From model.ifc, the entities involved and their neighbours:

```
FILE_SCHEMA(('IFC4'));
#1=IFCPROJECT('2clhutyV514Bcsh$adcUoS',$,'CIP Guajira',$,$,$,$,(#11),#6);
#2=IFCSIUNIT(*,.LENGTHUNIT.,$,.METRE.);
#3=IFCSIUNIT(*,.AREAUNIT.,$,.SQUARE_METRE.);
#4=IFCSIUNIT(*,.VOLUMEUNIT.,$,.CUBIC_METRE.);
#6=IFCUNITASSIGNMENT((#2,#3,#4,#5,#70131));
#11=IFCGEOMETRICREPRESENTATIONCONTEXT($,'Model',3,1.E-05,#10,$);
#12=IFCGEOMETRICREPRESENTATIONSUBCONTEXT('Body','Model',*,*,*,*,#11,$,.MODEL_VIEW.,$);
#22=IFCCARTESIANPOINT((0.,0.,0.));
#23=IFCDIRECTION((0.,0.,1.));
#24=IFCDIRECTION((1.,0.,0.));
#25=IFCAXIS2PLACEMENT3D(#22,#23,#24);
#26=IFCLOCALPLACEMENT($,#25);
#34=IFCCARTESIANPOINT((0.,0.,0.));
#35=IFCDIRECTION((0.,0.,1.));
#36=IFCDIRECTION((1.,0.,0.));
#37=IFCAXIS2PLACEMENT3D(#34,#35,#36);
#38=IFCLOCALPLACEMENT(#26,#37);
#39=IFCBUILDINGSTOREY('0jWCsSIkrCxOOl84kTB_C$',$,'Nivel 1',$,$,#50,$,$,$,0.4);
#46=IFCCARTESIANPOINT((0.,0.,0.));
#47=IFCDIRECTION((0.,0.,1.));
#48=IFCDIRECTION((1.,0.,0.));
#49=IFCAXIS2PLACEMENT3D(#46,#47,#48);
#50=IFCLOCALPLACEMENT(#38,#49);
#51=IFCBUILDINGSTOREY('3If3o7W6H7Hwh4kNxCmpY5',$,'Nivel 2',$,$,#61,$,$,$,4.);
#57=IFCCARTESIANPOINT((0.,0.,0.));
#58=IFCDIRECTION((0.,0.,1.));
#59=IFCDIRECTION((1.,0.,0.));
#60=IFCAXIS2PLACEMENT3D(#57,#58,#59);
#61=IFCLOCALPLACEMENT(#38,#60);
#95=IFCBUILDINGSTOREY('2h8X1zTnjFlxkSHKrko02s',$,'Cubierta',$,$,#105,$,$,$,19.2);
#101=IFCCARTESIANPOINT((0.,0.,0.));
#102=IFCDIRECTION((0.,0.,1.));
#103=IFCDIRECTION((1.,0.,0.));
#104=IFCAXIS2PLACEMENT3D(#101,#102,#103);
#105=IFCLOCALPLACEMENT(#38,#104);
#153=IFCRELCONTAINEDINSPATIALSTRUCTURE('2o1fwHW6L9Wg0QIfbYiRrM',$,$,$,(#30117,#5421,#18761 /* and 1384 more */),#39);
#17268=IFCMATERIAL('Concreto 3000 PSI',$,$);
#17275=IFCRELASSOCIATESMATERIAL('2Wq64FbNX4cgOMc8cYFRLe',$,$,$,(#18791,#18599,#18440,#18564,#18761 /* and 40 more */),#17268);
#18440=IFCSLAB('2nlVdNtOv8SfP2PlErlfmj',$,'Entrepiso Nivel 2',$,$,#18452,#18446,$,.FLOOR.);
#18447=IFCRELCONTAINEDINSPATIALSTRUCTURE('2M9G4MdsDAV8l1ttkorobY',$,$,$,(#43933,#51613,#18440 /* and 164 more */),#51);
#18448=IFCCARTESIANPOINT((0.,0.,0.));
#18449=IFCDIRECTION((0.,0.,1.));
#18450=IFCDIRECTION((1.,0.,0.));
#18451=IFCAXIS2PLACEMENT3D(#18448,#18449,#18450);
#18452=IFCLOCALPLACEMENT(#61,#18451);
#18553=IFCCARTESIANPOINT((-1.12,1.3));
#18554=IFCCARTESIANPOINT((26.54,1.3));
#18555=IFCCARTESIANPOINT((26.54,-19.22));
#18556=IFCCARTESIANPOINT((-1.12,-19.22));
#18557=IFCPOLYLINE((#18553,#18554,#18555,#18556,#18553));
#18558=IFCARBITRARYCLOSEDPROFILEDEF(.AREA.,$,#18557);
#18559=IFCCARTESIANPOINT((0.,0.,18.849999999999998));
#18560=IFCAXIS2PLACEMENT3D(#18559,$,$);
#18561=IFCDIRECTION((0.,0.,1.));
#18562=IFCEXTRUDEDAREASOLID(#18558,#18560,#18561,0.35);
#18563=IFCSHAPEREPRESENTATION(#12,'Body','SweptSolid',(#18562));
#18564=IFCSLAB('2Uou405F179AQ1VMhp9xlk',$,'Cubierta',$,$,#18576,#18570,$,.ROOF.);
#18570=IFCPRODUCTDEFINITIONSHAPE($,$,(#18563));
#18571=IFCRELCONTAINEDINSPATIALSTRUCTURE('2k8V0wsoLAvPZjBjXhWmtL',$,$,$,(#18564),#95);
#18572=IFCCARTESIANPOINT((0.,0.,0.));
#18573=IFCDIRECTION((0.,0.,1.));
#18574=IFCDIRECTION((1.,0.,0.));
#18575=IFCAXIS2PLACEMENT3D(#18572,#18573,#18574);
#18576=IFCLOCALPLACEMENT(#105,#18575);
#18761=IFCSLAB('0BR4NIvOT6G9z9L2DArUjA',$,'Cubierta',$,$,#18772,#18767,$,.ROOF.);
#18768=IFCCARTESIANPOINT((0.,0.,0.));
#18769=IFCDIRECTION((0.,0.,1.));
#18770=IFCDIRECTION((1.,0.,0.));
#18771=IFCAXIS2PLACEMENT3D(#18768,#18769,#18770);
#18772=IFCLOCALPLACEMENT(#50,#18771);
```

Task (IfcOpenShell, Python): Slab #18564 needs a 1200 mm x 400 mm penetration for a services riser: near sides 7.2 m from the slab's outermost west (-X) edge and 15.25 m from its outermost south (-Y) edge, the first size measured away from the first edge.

```python
import numpy as np
import ifcopenshell
import ifcopenshell.api.feature
import ifcopenshell.api.geometry
import ifcopenshell.api.root
import ifcopenshell.geom
import ifcopenshell.util.placement
import ifcopenshell.util.representation
import ifcopenshell.util.shape
import ifcopenshell.util.unit

model = ifcopenshell.open("model.ifc")
unit_scale = ifcopenshell.util.unit.calculate_unit_scale(model)
settings = ifcopenshell.geom.settings()


def volume(element):
    """Net volume in cubic metres, openings subtracted."""
    shape = ifcopenshell.geom.create_shape(settings, element)
    return ifcopenshell.util.shape.get_volume(shape.geometry)


slab = model.by_guid("2Uou405F179AQ1VMhp9xlk")
before = volume(slab)

# Extent in the slab's own axes, in metres. The edges named are its -X and -Y sides.
slab_shape = ifcopenshell.geom.create_shape(settings, slab)
vertices = ifcopenshell.util.shape.get_vertices(slab_shape.geometry)
x_min, y_min, bottom = vertices.min(axis=0)
top = vertices[:, 2].max()

opening = ifcopenshell.api.root.create_entity(model, ifc_class="IfcOpeningElement", name="Services riser opening", predefined_type="OPENING")
context = ifcopenshell.util.representation.get_context(model, "Model", "Body", "MODEL_VIEW")
width, depth = 1.2, 0.4
outline = [(0.0, 0.0), (width, 0.0), (width, depth), (0.0, depth), (0.0, 0.0)]
# Overshoot both faces by 50 mm so the cut is clean.
shape = ifcopenshell.api.geometry.add_slab_representation(
    model, context=context, depth=top - bottom + 0.1, polyline=outline
)
ifcopenshell.api.geometry.assign_representation(model, product=opening, representation=shape)

matrix = ifcopenshell.util.placement.get_local_placement(slab.ObjectPlacement)
matrix[:, 3] = matrix @ np.append(np.array([x_min + 7.2, y_min + 15.25, bottom - 0.05]) / unit_scale, 1.0)
ifcopenshell.api.geometry.edit_object_placement(model, product=opening, matrix=matrix, is_si=False)
ifcopenshell.api.feature.add_feature(model, feature=opening, element=slab)

after = volume(slab)

print(f"slab volume {before:.3f} -> {after:.3f} m3")

model.write("model_rev.ifc")
```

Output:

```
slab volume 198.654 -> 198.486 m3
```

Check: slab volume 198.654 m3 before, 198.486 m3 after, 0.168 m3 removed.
